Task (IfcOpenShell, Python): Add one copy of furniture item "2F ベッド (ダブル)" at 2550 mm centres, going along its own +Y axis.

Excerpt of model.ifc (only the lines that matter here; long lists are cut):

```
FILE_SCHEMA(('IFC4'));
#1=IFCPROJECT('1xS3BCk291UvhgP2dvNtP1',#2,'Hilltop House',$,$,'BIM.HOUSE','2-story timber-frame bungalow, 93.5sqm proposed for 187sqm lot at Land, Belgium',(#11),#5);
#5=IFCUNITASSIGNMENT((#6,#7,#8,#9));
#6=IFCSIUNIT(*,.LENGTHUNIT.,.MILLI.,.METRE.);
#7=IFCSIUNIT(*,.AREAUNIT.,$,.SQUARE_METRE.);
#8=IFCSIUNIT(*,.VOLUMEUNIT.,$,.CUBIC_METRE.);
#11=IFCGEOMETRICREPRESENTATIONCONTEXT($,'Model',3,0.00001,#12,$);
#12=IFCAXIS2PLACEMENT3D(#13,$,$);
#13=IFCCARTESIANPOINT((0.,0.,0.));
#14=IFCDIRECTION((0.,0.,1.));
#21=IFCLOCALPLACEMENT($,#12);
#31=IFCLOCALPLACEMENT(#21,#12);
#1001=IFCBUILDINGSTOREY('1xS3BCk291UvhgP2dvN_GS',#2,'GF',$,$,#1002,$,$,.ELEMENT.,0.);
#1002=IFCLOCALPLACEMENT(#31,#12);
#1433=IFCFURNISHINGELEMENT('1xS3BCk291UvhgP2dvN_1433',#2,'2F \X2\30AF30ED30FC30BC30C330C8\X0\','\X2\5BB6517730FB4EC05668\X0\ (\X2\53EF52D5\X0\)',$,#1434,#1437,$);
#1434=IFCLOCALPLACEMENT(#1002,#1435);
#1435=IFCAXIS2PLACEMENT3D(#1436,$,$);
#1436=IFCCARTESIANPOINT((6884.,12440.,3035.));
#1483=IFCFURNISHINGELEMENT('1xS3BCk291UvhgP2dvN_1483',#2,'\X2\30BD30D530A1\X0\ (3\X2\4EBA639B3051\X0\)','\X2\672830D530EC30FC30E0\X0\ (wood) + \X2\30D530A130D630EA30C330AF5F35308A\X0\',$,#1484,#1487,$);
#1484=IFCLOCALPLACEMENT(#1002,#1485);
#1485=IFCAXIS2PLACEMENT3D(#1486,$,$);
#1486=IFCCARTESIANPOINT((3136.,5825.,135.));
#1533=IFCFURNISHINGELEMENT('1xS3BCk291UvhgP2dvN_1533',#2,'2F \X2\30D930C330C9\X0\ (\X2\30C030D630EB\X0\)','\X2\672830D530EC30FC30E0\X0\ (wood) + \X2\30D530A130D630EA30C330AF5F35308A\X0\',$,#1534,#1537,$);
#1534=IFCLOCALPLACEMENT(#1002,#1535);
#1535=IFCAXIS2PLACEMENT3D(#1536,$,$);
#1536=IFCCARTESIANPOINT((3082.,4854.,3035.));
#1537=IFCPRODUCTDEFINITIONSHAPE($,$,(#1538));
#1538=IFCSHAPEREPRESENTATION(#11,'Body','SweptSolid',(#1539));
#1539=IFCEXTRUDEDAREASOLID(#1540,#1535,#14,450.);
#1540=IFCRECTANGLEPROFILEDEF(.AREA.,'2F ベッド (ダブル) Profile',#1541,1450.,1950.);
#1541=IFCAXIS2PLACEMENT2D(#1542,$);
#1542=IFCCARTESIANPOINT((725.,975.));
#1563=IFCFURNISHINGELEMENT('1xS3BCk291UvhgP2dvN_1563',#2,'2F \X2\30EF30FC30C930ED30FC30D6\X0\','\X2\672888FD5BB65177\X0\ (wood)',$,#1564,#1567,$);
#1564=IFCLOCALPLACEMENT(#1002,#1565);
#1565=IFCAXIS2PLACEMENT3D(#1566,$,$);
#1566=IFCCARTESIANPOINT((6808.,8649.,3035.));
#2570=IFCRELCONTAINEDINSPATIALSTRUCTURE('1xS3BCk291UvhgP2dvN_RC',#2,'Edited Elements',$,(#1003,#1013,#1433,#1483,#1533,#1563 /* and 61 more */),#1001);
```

```python
import ifcopenshell
import ifcopenshell.api.geometry
import ifcopenshell.api.root
import ifcopenshell.util.element
import ifcopenshell.util.placement
import ifcopenshell.util.unit

model = ifcopenshell.open("model.ifc")
unit_scale = ifcopenshell.util.unit.calculate_unit_scale(model)


def reuse_history(source, copy):
    """copy_class also copies each property set's owner history, people and application; keep the originals."""
    for rel in copy.IsDefinedBy:
        if rel.is_a("IfcRelDefinesByProperties") and (history := rel.RelatingPropertyDefinition.OwnerHistory):
            rel.RelatingPropertyDefinition.OwnerHistory = source.OwnerHistory
            ifcopenshell.util.element.remove_deep2(model, history)


source = model.by_guid("1xS3BCk291UvhgP2dvN_1533")
base = ifcopenshell.util.placement.get_local_placement(source.ObjectPlacement)
step = base[:3, 1] * 2.55 / unit_scale

for i in range(1, 2):
    copy = ifcopenshell.api.root.copy_class(model, product=source)
    copy.Representation = ifcopenshell.util.element.copy_deep(
        model, source.Representation, exclude=["IfcGeometricRepresentationContext", "IfcRepresentationMap"]
    )
    reuse_history(source, copy)
    matrix = base.copy()
    matrix[:3, 3] += i * step
    print("added at", matrix[:3, 3].round(3) + 0.0)
    ifcopenshell.api.geometry.edit_object_placement(model, product=copy, matrix=matrix, is_si=False)

model.write("model_v2.ifc")
```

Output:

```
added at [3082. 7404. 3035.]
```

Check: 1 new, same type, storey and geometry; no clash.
